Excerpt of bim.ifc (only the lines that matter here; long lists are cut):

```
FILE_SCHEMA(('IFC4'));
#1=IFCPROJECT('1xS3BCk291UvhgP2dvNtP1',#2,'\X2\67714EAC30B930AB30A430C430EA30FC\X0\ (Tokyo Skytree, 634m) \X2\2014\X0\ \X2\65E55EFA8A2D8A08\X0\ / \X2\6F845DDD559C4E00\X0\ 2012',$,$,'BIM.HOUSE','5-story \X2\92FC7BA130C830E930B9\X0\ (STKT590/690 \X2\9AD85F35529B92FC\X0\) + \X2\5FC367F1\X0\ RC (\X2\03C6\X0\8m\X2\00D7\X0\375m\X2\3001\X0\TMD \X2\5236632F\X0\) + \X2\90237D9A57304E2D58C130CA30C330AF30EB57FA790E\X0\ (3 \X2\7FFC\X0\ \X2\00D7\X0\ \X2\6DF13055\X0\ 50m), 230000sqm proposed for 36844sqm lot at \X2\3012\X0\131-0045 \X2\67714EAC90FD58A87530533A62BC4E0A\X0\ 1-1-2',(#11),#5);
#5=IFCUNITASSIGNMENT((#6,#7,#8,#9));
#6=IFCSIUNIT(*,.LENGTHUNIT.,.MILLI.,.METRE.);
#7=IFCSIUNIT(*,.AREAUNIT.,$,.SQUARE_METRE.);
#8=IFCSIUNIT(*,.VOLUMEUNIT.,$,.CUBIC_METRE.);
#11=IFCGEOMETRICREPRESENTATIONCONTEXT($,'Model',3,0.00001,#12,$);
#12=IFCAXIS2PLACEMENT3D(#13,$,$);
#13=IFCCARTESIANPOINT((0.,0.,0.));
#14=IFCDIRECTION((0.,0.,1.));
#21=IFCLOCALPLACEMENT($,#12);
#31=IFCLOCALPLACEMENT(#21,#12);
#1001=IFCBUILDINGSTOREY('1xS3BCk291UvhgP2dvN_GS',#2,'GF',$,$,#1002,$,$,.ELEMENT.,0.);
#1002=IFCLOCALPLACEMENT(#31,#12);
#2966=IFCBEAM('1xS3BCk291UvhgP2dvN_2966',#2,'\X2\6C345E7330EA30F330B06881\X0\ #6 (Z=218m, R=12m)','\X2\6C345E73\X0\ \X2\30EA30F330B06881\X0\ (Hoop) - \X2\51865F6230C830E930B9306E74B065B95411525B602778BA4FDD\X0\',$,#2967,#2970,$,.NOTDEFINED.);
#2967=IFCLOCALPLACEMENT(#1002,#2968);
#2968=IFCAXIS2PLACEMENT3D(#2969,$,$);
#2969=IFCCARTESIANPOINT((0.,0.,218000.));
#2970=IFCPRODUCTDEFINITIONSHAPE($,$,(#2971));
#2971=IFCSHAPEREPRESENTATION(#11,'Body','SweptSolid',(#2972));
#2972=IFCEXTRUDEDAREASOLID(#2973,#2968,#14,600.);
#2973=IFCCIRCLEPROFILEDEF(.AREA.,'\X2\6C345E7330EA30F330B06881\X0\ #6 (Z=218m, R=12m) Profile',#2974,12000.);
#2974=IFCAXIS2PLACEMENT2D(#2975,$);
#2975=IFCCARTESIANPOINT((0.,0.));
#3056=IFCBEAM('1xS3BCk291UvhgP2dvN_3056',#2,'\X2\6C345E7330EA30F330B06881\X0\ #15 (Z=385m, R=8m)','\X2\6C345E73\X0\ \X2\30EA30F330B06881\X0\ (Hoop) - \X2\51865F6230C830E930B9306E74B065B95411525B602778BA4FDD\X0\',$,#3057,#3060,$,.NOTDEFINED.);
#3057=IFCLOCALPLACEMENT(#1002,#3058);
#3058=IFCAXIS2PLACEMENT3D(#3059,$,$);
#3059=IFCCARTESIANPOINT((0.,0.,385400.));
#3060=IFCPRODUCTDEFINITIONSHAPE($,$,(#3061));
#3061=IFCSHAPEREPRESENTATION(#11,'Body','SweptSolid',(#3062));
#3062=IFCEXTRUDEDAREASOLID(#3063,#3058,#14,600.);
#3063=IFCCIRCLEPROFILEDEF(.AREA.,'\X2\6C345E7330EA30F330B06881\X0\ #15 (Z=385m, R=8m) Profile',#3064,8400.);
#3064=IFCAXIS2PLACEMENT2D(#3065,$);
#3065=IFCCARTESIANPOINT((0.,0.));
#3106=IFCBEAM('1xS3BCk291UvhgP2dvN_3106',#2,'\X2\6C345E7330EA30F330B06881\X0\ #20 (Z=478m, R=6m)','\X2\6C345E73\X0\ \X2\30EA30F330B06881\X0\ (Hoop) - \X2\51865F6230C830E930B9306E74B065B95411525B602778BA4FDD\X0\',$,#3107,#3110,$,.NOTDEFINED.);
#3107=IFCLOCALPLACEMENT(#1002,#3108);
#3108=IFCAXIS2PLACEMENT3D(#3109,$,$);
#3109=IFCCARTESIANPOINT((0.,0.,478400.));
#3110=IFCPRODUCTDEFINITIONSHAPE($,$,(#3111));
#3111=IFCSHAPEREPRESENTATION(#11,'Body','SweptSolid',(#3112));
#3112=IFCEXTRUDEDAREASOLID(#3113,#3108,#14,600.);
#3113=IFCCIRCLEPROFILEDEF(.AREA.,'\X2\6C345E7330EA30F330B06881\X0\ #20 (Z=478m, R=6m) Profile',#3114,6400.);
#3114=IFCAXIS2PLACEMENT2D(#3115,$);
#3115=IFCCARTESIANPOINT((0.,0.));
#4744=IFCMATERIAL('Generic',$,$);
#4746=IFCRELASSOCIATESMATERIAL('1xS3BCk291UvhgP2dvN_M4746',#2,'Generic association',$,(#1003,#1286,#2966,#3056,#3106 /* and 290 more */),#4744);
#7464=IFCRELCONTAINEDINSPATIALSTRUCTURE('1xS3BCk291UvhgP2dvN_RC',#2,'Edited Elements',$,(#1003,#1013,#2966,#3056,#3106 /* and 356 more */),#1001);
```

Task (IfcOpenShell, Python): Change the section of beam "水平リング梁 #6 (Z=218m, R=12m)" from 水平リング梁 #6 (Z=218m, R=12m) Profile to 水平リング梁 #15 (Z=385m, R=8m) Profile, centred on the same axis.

```python
import ifcopenshell
import ifcopenshell.util.element

model = ifcopenshell.open("bim.ifc")

member = model.by_id(2966)
source = next(p for p in model.by_type("IfcCircleProfileDef") if p.ProfileName == "水平リング梁 #15 (Z=385m, R=8m) Profile")

body = next(r for r in member.Representation.Representations if r.RepresentationIdentifier == "Body")
solid = body.Items[0]
old_profile = solid.SweptArea

# Copy the section's sizes but keep this member's own profile position.
profile = ifcopenshell.util.element.copy(model, source)
profile.Position = old_profile.Position
solid.SweptArea = profile
if not model.get_total_inverses(old_profile):
    ifcopenshell.util.element.remove_deep2(model, old_profile)

print(solid.SweptArea)

model.write("bim-out.ifc")
```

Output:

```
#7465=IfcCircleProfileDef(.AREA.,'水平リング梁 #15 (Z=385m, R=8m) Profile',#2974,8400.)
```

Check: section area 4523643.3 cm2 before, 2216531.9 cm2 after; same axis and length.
